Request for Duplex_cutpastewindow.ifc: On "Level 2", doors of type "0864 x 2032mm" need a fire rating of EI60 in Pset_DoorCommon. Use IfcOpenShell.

First a look at what the model holds.

```python
import ifcopenshell
import ifcopenshell.util.element

model = ifcopenshell.open("Duplex_cutpastewindow.ifc")
print(model.schema)
storey = next(s for s in model.by_type("IfcBuildingStorey") if s.Name == "Level 2")
doors = [e for e in ifcopenshell.util.element.get_decomposition(storey) if e.is_a("IfcDoor")]
seen = {}
for e in doors:
    element_type = ifcopenshell.util.element.get_type(e)
    key = (element_type.Name if element_type != e and element_type else None, ifcopenshell.util.element.get_pset(e, "Pset_DoorCommon", "FireRating"))
    seen[key] = seen.get(key, 0) + 1
for (name, value), count in sorted(seen.items(), key=str):
    print(count, "x", name, "|", value)
```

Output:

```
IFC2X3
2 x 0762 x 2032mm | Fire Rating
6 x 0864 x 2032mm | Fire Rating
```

```python
import ifcopenshell
import ifcopenshell.api.pset
import ifcopenshell.util.element

model = ifcopenshell.open("Duplex_cutpastewindow.ifc")

storey = next(s for s in model.by_type("IfcBuildingStorey") if s.Name == "Level 2")
doors = [e for e in ifcopenshell.util.element.get_decomposition(storey) if e.is_a("IfcDoor")]

count = 0
for e in doors:
    element_type = ifcopenshell.util.element.get_type(e)
    if element_type in (None, e) or element_type.Name != "0864 x 2032mm":
        continue
    # add_pset returns the element's existing set when there is one.
    pset = ifcopenshell.api.pset.add_pset(model, product=e, name="Pset_DoorCommon")
    ifcopenshell.api.pset.edit_pset(model, pset=pset, properties={"FireRating": "EI60"})
    count += 1

print(count, "doors updated")

model.write("Duplex_cutpastewindow_edited.ifc")
```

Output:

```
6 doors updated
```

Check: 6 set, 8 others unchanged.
